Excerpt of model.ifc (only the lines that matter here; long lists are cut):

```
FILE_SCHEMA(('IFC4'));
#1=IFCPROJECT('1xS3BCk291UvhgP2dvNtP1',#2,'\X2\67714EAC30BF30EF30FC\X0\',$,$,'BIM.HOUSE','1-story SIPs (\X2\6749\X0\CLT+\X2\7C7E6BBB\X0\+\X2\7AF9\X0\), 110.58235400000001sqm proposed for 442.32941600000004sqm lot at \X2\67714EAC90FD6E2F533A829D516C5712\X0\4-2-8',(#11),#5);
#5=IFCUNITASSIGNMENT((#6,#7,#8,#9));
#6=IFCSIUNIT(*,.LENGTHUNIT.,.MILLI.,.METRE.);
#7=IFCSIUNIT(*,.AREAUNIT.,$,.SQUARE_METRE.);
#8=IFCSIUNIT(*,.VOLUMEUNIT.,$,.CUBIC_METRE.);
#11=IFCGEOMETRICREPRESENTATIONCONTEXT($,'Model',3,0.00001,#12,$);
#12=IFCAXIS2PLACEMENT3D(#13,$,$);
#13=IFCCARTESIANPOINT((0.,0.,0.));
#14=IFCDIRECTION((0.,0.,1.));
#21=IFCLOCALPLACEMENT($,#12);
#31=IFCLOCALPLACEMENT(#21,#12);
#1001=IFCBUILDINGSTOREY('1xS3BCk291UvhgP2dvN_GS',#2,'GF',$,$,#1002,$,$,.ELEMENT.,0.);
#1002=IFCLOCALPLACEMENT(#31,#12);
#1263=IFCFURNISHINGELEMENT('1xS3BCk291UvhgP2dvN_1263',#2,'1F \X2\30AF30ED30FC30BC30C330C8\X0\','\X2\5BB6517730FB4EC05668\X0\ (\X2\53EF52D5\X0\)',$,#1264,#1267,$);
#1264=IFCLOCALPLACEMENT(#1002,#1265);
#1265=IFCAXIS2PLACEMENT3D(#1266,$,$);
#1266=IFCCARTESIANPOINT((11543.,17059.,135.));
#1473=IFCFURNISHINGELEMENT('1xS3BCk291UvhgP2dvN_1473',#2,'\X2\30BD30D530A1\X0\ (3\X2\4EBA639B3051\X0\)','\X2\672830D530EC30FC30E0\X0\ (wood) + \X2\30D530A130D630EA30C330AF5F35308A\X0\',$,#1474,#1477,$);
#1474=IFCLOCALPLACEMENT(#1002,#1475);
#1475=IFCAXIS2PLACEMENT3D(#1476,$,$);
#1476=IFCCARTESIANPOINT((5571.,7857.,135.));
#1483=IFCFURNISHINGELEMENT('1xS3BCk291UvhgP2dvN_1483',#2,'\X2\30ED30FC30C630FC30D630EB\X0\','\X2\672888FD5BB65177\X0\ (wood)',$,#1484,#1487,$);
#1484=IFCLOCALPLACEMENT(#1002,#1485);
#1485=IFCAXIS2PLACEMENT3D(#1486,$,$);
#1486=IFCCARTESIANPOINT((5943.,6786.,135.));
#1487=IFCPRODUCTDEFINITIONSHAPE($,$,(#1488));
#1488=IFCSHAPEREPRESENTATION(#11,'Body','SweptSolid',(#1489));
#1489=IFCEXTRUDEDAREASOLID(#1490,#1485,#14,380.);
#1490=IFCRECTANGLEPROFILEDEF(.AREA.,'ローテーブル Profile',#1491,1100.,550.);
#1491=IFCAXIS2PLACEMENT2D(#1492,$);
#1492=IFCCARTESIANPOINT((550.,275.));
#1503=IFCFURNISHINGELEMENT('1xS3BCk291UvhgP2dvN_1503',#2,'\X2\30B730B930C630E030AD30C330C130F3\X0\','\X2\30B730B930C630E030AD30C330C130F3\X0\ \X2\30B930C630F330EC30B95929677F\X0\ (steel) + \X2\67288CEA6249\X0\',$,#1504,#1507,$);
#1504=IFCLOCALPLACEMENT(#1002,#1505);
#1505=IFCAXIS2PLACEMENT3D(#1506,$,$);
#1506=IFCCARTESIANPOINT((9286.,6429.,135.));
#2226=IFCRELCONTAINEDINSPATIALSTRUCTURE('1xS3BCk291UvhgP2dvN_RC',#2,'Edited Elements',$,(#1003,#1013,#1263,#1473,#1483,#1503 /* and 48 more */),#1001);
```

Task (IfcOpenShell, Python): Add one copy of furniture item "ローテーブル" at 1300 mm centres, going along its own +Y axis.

```python
import ifcopenshell
import ifcopenshell.api.geometry
import ifcopenshell.api.root
import ifcopenshell.util.element
import ifcopenshell.util.placement
import ifcopenshell.util.unit

model = ifcopenshell.open("model.ifc")
unit_scale = ifcopenshell.util.unit.calculate_unit_scale(model)


def reuse_history(source, copy):
    """copy_class also copies each property set's owner history, people and application; keep the originals."""
    for rel in copy.IsDefinedBy:
        if rel.is_a("IfcRelDefinesByProperties") and (history := rel.RelatingPropertyDefinition.OwnerHistory):
            rel.RelatingPropertyDefinition.OwnerHistory = source.OwnerHistory
            ifcopenshell.util.element.remove_deep2(model, history)


source = model.by_id(1483)
base = ifcopenshell.util.placement.get_local_placement(source.ObjectPlacement)
step = base[:3, 1] * 1.3 / unit_scale

for i in range(1, 2):
    copy = ifcopenshell.api.root.copy_class(model, product=source)
    copy.Representation = ifcopenshell.util.element.copy_deep(
        model, source.Representation, exclude=["IfcGeometricRepresentationContext", "IfcRepresentationMap"]
    )
    reuse_history(source, copy)
    matrix = base.copy()
    matrix[:3, 3] += i * step
    print("added at", matrix[:3, 3].round(3) + 0.0)
    ifcopenshell.api.geometry.edit_object_placement(model, product=copy, matrix=matrix, is_si=False)

model.write("model_rev.ifc")
```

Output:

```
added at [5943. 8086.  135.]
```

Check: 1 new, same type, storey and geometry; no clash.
